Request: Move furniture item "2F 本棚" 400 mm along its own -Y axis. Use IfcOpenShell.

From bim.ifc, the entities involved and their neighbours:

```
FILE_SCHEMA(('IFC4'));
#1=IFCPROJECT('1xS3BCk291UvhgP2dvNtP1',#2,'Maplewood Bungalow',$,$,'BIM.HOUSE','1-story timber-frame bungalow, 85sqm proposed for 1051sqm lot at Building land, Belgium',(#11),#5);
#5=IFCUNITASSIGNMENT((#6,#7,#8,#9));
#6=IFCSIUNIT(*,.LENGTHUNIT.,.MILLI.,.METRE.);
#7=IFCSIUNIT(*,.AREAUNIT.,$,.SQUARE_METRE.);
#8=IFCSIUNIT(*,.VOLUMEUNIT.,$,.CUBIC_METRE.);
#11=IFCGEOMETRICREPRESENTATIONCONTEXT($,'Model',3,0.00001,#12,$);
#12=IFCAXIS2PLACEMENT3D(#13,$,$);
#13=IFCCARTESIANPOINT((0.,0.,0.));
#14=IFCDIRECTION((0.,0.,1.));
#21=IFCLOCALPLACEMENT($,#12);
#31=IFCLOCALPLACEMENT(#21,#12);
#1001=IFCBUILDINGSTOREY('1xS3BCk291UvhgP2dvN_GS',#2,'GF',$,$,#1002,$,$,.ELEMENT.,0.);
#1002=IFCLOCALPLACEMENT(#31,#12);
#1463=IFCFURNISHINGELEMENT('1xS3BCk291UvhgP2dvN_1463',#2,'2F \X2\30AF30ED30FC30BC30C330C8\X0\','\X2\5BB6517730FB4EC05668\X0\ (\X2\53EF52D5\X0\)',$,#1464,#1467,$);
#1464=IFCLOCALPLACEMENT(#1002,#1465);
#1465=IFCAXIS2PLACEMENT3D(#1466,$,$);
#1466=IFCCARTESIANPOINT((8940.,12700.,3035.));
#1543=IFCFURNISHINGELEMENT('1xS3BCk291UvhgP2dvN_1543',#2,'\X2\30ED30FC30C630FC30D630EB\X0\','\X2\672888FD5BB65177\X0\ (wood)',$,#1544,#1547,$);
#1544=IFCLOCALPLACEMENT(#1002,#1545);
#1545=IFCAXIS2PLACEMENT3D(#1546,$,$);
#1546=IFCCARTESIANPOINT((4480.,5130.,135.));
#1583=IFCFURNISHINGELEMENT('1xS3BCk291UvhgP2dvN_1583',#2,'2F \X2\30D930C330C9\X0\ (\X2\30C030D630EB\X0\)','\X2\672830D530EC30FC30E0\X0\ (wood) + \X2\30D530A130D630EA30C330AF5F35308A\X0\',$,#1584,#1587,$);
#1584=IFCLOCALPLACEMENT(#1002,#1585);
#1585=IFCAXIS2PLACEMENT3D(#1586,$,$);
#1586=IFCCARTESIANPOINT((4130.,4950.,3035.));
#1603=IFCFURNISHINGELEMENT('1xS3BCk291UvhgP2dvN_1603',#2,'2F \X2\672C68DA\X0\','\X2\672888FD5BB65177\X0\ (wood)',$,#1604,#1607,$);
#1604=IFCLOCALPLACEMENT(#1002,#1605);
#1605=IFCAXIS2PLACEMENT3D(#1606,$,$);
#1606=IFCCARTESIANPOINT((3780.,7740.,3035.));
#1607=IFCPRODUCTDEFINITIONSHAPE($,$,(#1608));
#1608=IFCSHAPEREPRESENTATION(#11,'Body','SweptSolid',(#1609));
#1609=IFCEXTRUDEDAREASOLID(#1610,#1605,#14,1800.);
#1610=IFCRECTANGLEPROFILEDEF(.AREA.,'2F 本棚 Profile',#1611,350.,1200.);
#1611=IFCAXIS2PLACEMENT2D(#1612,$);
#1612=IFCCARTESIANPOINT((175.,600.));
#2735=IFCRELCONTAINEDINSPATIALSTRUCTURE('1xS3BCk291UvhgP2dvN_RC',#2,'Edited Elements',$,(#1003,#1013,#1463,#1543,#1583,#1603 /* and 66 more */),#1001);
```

```python
import ifcopenshell
import ifcopenshell.api.geometry
import ifcopenshell.util.placement
import ifcopenshell.util.unit

model = ifcopenshell.open("bim.ifc")
unit_scale = ifcopenshell.util.unit.calculate_unit_scale(model)

item = model.by_guid("1xS3BCk291UvhgP2dvN_1603")
matrix = ifcopenshell.util.placement.get_local_placement(item.ObjectPlacement)
matrix[:3, 3] -= matrix[:3, 1] * 0.4 / unit_scale
ifcopenshell.api.geometry.edit_object_placement(model, product=item, matrix=matrix, is_si=False)

print(ifcopenshell.util.placement.get_local_placement(item.ObjectPlacement).round(3) + 0.0)

model.write("bim-out.ifc")
```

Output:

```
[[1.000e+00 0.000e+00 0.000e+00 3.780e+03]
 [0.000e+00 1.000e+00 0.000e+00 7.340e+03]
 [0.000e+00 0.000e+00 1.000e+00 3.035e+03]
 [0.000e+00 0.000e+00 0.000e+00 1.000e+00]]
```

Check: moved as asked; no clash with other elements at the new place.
